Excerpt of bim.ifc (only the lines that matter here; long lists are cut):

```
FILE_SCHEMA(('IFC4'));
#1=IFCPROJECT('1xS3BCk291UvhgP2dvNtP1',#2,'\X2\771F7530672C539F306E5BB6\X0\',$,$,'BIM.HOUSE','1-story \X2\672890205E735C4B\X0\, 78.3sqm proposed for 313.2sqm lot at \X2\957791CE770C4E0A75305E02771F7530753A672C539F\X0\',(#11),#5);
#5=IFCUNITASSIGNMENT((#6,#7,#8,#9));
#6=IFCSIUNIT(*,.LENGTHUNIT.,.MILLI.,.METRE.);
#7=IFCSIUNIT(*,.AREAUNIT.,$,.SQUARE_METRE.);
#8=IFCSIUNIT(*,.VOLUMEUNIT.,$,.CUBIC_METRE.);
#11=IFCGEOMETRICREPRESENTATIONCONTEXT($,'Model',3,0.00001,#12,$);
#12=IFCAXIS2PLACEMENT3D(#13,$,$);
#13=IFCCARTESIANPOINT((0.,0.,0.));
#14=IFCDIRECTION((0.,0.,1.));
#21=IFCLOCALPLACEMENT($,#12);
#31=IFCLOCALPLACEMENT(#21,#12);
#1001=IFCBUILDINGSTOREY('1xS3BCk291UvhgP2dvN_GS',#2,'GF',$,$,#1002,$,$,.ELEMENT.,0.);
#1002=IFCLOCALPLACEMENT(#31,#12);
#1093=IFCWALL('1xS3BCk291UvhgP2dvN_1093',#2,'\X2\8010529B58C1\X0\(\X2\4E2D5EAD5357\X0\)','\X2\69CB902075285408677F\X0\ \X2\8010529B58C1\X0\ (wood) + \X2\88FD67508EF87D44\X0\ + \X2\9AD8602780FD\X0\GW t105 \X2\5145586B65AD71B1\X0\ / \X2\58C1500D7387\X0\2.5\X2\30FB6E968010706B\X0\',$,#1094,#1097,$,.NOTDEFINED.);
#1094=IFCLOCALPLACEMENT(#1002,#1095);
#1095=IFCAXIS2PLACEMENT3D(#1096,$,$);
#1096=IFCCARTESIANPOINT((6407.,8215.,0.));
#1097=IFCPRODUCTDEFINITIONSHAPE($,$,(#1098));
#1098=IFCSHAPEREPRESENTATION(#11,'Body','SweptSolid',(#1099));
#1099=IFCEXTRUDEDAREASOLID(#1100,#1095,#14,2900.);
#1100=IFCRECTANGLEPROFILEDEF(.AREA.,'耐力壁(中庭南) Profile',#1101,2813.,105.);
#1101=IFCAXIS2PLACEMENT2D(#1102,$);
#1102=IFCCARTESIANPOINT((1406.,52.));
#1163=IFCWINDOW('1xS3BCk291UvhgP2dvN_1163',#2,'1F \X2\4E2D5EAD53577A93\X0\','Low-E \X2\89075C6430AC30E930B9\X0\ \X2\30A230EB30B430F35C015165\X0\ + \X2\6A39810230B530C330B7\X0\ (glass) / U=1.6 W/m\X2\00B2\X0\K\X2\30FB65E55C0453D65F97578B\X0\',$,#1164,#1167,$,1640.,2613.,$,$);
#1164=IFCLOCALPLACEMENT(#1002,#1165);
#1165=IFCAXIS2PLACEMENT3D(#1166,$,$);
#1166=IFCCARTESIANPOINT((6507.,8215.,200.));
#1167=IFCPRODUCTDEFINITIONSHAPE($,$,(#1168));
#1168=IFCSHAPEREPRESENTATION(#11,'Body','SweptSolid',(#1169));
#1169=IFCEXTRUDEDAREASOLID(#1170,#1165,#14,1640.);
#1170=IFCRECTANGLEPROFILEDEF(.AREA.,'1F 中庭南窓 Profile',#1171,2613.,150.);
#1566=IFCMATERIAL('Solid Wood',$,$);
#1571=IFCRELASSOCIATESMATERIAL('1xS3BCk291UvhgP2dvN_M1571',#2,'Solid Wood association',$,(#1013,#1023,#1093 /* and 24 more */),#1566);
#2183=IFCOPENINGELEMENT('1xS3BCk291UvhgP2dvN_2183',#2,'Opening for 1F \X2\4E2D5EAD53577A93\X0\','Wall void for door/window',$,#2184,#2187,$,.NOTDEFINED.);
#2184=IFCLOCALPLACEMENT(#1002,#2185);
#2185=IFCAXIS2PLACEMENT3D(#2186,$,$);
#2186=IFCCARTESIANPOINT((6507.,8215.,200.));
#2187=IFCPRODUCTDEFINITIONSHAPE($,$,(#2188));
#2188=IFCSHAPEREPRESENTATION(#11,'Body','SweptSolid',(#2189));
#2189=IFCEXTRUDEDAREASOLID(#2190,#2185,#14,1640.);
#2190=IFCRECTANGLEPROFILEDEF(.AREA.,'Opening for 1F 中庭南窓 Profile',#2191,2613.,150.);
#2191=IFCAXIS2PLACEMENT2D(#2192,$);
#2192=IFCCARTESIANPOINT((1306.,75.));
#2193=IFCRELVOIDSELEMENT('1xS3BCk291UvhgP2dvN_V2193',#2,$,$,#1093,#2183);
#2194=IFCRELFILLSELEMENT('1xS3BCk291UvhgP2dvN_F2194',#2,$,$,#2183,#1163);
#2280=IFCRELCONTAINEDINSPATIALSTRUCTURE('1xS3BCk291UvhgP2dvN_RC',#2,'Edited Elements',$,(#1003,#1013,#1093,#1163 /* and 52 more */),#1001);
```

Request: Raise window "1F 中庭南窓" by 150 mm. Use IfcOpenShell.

```python
import numpy as np
import ifcopenshell
import ifcopenshell.api.geometry
import ifcopenshell.util.placement
import ifcopenshell.util.unit

model = ifcopenshell.open("bim.ifc")
unit_scale = ifcopenshell.util.unit.calculate_unit_scale(model)

window = model.by_id(1163)
opening = window.FillsVoids[0].RelatingOpeningElement
dz = 0.15 / unit_scale

shift = np.array([0.0, 0.0, dz])
# The window is not placed relative to its opening, so move both.
for product in (opening, window):
    matrix = ifcopenshell.util.placement.get_local_placement(product.ObjectPlacement)
    matrix[:3, 3] += shift
    ifcopenshell.api.geometry.edit_object_placement(model, product=product, matrix=matrix, is_si=False)

print(f"moved by {dz * unit_scale:+.3f} m")

model.write("bim_v2.ifc")
```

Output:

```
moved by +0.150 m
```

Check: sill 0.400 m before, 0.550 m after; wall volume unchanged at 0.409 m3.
